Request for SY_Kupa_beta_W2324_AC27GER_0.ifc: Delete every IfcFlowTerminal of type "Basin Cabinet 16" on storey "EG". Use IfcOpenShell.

First a look at what the model holds.

```python
import ifcopenshell
import ifcopenshell.util.element

model = ifcopenshell.open("SY_Kupa_beta_W2324_AC27GER_0.ifc")
print(model.schema)
storey = next(s for s in model.by_type("IfcBuildingStorey") if s.Name == "EG")
terminals = [e for e in ifcopenshell.util.element.get_decomposition(storey) if e.is_a("IfcFlowTerminal")]
seen = {}
for e in terminals:
    element_type = ifcopenshell.util.element.get_type(e)
    name = element_type.Name if element_type not in (None, e) else None
    seen[name] = seen.get(name, 0) + 1
for name, count in sorted(seen.items(), key=str):
    print(count, "x", name)
```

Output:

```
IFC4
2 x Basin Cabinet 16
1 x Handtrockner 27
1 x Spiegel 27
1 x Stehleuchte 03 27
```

```python
import ifcopenshell
import ifcopenshell.api.root
import ifcopenshell.util.element

model = ifcopenshell.open("SY_Kupa_beta_W2324_AC27GER_0.ifc")

storey = next(s for s in model.by_type("IfcBuildingStorey") if s.Name == "EG")
terminals = [e for e in ifcopenshell.util.element.get_decomposition(storey) if e.is_a("IfcFlowTerminal")]
targets = [e for e in terminals if (t := ifcopenshell.util.element.get_type(e)) not in (None, e) and t.Name == "Basin Cabinet 16"]

for e in targets:
    ifcopenshell.api.root.remove_product(model, product=e)
print(len(targets), "removed")

model.write("SY_Kupa_beta_W2324_AC27GER_0_rev.ifc")
```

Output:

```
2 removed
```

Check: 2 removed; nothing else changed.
